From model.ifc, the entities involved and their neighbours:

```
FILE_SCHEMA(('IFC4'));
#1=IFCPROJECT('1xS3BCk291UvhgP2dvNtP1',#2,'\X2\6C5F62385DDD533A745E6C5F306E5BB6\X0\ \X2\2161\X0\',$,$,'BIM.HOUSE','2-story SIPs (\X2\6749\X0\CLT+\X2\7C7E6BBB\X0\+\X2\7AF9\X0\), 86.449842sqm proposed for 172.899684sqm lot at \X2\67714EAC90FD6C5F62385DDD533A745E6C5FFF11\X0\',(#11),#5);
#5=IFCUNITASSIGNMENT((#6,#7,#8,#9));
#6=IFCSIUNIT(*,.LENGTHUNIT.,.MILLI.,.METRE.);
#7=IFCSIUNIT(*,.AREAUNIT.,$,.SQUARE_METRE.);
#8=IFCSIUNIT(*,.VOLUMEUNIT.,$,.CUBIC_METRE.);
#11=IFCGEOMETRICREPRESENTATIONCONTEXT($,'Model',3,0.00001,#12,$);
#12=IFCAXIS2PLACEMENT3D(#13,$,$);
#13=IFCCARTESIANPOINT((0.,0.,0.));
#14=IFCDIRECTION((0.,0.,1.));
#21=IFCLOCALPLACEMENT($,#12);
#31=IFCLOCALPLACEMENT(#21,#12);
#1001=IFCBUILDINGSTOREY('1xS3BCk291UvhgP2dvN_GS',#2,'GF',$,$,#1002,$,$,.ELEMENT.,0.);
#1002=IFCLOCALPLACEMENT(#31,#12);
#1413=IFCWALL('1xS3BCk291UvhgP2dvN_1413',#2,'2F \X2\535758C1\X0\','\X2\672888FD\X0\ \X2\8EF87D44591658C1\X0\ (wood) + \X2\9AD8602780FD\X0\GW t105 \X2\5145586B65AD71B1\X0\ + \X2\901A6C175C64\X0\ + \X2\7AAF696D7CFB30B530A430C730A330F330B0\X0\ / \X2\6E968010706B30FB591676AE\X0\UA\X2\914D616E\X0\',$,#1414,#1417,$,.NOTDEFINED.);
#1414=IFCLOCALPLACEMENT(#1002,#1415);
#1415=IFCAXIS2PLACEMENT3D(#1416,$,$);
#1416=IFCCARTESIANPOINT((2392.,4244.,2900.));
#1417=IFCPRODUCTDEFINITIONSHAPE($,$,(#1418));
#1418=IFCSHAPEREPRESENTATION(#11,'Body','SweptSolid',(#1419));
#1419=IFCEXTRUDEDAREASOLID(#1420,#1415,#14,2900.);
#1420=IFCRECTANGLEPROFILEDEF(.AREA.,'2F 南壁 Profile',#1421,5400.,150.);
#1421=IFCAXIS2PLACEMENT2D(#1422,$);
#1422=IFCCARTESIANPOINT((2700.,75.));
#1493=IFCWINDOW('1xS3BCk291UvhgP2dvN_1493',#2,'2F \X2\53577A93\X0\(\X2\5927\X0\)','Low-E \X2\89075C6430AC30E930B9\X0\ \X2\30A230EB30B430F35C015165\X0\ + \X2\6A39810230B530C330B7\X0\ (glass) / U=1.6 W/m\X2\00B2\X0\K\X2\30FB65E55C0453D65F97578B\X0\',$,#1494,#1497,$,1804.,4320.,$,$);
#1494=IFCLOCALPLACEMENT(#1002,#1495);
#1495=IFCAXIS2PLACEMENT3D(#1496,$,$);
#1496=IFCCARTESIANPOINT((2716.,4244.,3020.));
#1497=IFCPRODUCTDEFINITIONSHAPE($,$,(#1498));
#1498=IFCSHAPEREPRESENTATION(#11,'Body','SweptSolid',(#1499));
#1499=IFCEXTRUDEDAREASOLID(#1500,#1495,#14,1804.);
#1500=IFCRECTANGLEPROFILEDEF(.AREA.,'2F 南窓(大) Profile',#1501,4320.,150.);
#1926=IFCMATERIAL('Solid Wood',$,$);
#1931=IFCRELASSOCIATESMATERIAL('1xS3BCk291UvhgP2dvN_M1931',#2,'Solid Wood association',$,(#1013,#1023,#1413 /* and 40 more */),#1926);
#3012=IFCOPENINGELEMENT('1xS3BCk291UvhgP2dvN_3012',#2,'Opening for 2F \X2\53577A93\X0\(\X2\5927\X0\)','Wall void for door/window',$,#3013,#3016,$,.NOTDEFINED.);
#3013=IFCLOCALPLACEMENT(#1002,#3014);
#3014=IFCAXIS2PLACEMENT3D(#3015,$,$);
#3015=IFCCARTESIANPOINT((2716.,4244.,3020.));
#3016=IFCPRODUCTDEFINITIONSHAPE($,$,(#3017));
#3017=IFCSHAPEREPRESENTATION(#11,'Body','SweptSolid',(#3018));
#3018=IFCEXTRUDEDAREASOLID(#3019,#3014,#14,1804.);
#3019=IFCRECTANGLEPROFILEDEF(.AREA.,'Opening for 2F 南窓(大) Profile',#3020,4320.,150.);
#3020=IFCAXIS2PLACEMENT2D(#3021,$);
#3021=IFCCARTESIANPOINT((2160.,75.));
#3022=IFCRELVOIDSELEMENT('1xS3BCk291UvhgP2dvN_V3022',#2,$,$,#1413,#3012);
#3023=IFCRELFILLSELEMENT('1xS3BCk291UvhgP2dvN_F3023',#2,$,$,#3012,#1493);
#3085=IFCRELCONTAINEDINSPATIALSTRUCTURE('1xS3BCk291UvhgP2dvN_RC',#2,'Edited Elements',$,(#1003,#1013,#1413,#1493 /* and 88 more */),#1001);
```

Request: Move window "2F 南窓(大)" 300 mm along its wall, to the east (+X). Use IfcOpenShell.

```python
import ifcopenshell
import ifcopenshell.api.geometry
import ifcopenshell.util.placement
import ifcopenshell.util.unit

model = ifcopenshell.open("model.ifc")
unit_scale = ifcopenshell.util.unit.calculate_unit_scale(model)

window = model.by_guid("1xS3BCk291UvhgP2dvN_1493")
opening = window.FillsVoids[0].RelatingOpeningElement
wall = opening.VoidsElements[0].RelatingBuildingElement

wall_matrix = ifcopenshell.util.placement.get_local_placement(wall.ObjectPlacement)
shift = wall_matrix[:3, 0] * 0.3 / unit_scale
before = ifcopenshell.util.placement.get_local_placement(window.ObjectPlacement)[:3, 3].copy()

# The window is not placed relative to its opening, so move both.
for product in (opening, window):
    matrix = ifcopenshell.util.placement.get_local_placement(product.ObjectPlacement)
    matrix[:3, 3] += shift
    ifcopenshell.api.geometry.edit_object_placement(model, product=product, matrix=matrix, is_si=False)

after = ifcopenshell.util.placement.get_local_placement(window.ObjectPlacement)[:3, 3]
print("window moved by", (after - before).round(3) + 0.0)

model.write("model_rev.ifc")
```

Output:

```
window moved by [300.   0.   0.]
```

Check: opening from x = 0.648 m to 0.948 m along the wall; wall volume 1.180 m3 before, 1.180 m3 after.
